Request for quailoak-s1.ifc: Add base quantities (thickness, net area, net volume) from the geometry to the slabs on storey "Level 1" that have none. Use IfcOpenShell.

First a look at what the model holds.

```python
import ifcopenshell
import ifcopenshell.util.element
import ifcopenshell.util.unit

model = ifcopenshell.open("quailoak-s1.ifc")
print(model.schema)
for unit_type in ("LENGTHUNIT", "AREAUNIT", "VOLUMEUNIT"):
    print(unit_type, ifcopenshell.util.unit.calculate_unit_scale(model, unit_type))
storey = next(s for s in model.by_type("IfcBuildingStorey") if s.Name == "Level 1")
slabs = [e for e in ifcopenshell.util.element.get_decomposition(storey) if e.is_a("IfcSlab")]
for e in sorted(slabs, key=lambda e: e.id()):
    print(e.id(), e.is_a(), e.Name, list(ifcopenshell.util.element.get_psets(e, qtos_only=True)), sep=" | ")
```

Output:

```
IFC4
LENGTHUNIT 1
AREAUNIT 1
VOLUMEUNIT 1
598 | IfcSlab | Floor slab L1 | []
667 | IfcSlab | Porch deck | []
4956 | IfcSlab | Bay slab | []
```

```python
import ifcopenshell
import ifcopenshell.api.pset
import ifcopenshell.geom
import ifcopenshell.util.element
import ifcopenshell.util.shape
import ifcopenshell.util.unit

model = ifcopenshell.open("quailoak-s1.ifc")
unit_scale = ifcopenshell.util.unit.calculate_unit_scale(model)
area_scale = ifcopenshell.util.unit.calculate_unit_scale(model, "AREAUNIT")
volume_scale = ifcopenshell.util.unit.calculate_unit_scale(model, "VOLUMEUNIT")
settings = ifcopenshell.geom.settings()

storey = next(s for s in model.by_type("IfcBuildingStorey") if s.Name == "Level 1")
slabs = [e for e in ifcopenshell.util.element.get_decomposition(storey) if e.is_a("IfcSlab")]

for e in sorted(slabs, key=lambda e: e.id()):
    if ifcopenshell.util.element.get_psets(e, qtos_only=True, should_inherit=False):
        continue
    # Geometry comes back in metres, in the element's own axes.
    shape = ifcopenshell.geom.create_shape(settings, e)
    values = {
        "Width": ifcopenshell.util.shape.get_z(shape.geometry) / unit_scale,
        "NetArea": ifcopenshell.util.shape.get_footprint_area(shape.geometry) / area_scale,
        "NetVolume": ifcopenshell.util.shape.get_volume(shape.geometry) / volume_scale,
    }
    qto = ifcopenshell.api.pset.add_qto(model, product=e, name="Qto_SlabBaseQuantities")
    ifcopenshell.api.pset.edit_qto(model, qto=qto, properties=values)
    print(e.id(), {k: round(v, 3) for k, v in values.items()})

model.write("quailoak-s1_updated.ifc")
```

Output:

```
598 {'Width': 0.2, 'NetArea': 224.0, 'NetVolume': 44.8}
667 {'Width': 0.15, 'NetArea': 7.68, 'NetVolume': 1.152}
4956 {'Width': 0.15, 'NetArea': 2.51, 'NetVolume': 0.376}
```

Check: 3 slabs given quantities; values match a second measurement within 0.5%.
